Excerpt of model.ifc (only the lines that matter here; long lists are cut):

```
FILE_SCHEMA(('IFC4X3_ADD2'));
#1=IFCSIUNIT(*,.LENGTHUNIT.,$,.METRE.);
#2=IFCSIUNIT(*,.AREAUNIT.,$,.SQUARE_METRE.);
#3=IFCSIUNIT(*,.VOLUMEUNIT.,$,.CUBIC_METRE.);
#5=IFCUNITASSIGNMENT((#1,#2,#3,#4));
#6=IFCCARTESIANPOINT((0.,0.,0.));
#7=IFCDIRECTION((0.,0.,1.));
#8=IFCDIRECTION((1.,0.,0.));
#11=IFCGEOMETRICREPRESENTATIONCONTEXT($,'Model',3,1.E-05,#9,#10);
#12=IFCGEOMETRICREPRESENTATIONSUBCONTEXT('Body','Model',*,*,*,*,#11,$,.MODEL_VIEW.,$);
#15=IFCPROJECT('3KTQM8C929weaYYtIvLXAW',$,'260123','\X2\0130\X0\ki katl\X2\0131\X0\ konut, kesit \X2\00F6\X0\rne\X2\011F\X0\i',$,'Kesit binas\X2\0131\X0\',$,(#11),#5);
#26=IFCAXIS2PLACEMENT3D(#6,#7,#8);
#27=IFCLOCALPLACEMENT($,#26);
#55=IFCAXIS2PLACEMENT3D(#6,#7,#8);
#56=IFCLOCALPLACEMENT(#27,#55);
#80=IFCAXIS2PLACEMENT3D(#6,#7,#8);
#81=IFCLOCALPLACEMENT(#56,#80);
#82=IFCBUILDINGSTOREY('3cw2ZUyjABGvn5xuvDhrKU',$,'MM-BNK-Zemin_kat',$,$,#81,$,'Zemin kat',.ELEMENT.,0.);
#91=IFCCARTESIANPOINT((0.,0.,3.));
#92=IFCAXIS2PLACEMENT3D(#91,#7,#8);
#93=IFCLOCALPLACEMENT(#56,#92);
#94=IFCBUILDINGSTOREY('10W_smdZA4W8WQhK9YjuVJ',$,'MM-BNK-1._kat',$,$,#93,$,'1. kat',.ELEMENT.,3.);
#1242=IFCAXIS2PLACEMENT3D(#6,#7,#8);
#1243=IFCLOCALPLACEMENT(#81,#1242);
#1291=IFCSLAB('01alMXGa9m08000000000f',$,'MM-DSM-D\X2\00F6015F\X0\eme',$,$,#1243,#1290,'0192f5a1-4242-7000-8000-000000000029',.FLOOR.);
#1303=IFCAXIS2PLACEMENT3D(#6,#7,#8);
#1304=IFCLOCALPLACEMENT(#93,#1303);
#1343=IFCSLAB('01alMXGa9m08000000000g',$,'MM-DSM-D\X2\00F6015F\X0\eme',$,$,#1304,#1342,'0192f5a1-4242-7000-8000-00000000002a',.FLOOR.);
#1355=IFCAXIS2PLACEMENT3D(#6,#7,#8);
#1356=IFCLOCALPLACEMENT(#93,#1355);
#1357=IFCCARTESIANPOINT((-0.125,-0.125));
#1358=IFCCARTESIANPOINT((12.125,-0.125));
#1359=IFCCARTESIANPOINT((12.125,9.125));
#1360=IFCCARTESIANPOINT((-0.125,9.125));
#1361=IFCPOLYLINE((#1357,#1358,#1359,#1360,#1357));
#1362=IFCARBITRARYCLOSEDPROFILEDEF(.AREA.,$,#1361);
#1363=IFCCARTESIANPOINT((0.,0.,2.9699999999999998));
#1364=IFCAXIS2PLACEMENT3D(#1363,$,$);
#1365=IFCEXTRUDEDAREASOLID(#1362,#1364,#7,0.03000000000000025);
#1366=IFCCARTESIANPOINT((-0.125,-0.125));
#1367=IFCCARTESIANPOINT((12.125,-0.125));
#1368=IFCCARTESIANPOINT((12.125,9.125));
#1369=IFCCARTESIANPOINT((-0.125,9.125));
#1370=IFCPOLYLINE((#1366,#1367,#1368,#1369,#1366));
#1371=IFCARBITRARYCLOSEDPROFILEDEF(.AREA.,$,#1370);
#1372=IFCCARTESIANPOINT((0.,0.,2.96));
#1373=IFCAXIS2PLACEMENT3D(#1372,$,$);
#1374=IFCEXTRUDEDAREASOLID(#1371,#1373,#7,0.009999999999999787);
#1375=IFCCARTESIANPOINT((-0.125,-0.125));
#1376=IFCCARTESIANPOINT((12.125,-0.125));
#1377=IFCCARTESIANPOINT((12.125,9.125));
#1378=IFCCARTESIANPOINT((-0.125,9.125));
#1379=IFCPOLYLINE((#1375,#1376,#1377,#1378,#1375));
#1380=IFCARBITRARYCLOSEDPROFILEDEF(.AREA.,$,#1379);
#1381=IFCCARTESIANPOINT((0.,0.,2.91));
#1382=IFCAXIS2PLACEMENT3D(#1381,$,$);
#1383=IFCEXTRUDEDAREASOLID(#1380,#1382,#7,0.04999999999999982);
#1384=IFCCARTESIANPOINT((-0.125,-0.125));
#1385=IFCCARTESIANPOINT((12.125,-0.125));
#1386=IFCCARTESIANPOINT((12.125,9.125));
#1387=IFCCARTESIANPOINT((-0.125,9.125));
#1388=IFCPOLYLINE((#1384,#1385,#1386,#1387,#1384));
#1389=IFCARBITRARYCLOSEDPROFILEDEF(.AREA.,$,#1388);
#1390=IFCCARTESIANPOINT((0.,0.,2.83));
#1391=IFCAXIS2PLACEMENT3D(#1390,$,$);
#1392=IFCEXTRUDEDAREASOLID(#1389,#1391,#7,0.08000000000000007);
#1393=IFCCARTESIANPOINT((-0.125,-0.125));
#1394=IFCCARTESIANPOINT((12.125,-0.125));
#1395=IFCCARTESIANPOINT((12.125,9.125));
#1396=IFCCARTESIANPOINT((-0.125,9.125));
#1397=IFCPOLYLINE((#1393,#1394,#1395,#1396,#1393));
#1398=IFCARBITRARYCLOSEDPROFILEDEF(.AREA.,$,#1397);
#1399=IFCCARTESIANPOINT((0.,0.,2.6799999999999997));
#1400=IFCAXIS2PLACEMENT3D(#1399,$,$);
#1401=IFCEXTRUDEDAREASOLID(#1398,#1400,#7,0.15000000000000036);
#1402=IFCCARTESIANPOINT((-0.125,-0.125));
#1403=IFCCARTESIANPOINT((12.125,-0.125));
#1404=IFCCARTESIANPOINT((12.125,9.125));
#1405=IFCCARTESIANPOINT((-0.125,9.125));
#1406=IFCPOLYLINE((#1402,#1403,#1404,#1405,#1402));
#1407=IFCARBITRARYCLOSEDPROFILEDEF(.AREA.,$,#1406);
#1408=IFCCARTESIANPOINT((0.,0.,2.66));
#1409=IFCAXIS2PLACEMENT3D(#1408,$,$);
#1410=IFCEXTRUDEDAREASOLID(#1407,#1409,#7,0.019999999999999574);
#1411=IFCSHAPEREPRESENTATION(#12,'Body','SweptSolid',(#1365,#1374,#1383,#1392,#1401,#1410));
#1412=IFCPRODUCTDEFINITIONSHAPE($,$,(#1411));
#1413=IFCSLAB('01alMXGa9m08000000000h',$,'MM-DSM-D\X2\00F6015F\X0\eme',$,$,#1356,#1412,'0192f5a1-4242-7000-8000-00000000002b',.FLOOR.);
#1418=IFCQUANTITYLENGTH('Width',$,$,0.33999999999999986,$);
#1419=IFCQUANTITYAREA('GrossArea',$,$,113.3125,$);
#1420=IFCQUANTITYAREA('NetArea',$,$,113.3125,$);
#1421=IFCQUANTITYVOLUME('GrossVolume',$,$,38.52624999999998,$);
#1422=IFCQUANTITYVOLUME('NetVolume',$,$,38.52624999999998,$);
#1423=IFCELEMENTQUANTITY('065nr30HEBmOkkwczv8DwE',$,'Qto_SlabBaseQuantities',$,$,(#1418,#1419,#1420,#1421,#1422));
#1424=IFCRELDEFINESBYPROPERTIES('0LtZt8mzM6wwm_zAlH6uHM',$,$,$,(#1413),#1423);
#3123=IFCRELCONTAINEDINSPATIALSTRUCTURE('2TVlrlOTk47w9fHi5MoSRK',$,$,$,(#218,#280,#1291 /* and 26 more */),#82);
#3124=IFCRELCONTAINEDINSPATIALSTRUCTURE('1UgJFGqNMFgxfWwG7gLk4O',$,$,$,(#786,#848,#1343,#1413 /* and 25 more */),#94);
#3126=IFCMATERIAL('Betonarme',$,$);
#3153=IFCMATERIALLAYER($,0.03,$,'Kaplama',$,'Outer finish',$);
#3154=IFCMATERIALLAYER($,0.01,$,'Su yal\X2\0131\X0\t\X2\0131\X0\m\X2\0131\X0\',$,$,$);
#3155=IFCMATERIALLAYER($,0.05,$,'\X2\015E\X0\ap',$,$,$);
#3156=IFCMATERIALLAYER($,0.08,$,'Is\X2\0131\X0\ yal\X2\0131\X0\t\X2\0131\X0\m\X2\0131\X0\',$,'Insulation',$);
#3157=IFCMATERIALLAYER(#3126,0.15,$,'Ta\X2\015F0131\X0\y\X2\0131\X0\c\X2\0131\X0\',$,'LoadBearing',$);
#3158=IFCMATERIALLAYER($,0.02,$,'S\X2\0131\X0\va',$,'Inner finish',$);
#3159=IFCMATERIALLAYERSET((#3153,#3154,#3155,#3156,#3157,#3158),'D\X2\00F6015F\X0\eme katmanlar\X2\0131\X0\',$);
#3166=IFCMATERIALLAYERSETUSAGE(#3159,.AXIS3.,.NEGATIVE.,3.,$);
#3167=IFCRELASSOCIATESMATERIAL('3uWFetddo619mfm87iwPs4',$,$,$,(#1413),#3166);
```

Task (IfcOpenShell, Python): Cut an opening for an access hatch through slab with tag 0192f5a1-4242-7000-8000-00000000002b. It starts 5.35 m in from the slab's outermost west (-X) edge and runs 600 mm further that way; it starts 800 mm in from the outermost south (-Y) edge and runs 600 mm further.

```python
import numpy as np
import ifcopenshell
import ifcopenshell.api.feature
import ifcopenshell.api.geometry
import ifcopenshell.api.pset
import ifcopenshell.api.root
import ifcopenshell.geom
import ifcopenshell.util.element
import ifcopenshell.util.placement
import ifcopenshell.util.representation
import ifcopenshell.util.shape
import ifcopenshell.util.unit

model = ifcopenshell.open("model.ifc")
unit_scale = ifcopenshell.util.unit.calculate_unit_scale(model)
area_scale = ifcopenshell.util.unit.calculate_unit_scale(model, "AREAUNIT")
volume_scale = ifcopenshell.util.unit.calculate_unit_scale(model, "VOLUMEUNIT")
settings = ifcopenshell.geom.settings()


def volume(element):
    """Net volume in cubic metres, openings subtracted."""
    shape = ifcopenshell.geom.create_shape(settings, element)
    return ifcopenshell.util.shape.get_volume(shape.geometry)


slab = model.by_guid("01alMXGa9m08000000000h")
before = volume(slab)

# Extent in the slab's own axes, in metres. The edges named are its -X and -Y sides.
slab_shape = ifcopenshell.geom.create_shape(settings, slab)
vertices = ifcopenshell.util.shape.get_vertices(slab_shape.geometry)
x_min, y_min, bottom = vertices.min(axis=0)
top = vertices[:, 2].max()

opening = ifcopenshell.api.root.create_entity(model, ifc_class="IfcOpeningElement", name="Access hatch opening", predefined_type="OPENING")
context = ifcopenshell.util.representation.get_context(model, "Model", "Body", "MODEL_VIEW")
width, depth = 0.6, 0.6
outline = [(0.0, 0.0), (width, 0.0), (width, depth), (0.0, depth), (0.0, 0.0)]
# Overshoot both faces by 50 mm so the cut is clean.
shape = ifcopenshell.api.geometry.add_slab_representation(
    model, context=context, depth=top - bottom + 0.1, polyline=outline
)
ifcopenshell.api.geometry.assign_representation(model, product=opening, representation=shape)

matrix = ifcopenshell.util.placement.get_local_placement(slab.ObjectPlacement)
matrix[:, 3] = matrix @ np.append(np.array([x_min + 5.35, y_min + 0.8, bottom - 0.05]) / unit_scale, 1.0)
ifcopenshell.api.geometry.edit_object_placement(model, product=opening, matrix=matrix, is_si=False)
ifcopenshell.api.feature.add_feature(model, feature=opening, element=slab)

after = volume(slab)

# Update the slab's stored quantities.
qto = model.by_id(ifcopenshell.util.element.get_pset(slab, "Qto_SlabBaseQuantities", should_inherit=False)["id"])
ifcopenshell.api.pset.edit_qto(model, qto=qto, properties={
    "NetArea": after / (top - bottom) / area_scale,
    "NetVolume": after / volume_scale,
})

print(f"slab volume {before:.3f} -> {after:.3f} m3")

model.write("model_rev.ifc")
```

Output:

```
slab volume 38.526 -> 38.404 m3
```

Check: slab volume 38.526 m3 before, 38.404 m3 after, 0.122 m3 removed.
